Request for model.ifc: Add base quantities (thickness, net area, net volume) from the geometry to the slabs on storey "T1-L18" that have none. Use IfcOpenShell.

First a look at what the model holds.

```python
import ifcopenshell
import ifcopenshell.util.element
import ifcopenshell.util.unit

model = ifcopenshell.open("model.ifc")
print(model.schema)
for unit_type in ("LENGTHUNIT", "AREAUNIT", "VOLUMEUNIT"):
    print(unit_type, ifcopenshell.util.unit.calculate_unit_scale(model, unit_type))
storey = next(s for s in model.by_type("IfcBuildingStorey") if s.Name == "T1-L18")
slabs = [e for e in ifcopenshell.util.element.get_decomposition(storey) if e.is_a("IfcSlab")]
for e in sorted(slabs, key=lambda e: e.id()):
    print(e.id(), e.is_a(), e.Name, list(ifcopenshell.util.element.get_psets(e, qtos_only=True)), sep=" | ")
```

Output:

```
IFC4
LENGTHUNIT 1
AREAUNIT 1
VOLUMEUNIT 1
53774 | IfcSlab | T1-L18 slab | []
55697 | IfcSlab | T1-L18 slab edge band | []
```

```python
import ifcopenshell
import ifcopenshell.api.pset
import ifcopenshell.geom
import ifcopenshell.util.element
import ifcopenshell.util.shape
import ifcopenshell.util.unit

model = ifcopenshell.open("model.ifc")
unit_scale = ifcopenshell.util.unit.calculate_unit_scale(model)
area_scale = ifcopenshell.util.unit.calculate_unit_scale(model, "AREAUNIT")
volume_scale = ifcopenshell.util.unit.calculate_unit_scale(model, "VOLUMEUNIT")
settings = ifcopenshell.geom.settings()

storey = next(s for s in model.by_type("IfcBuildingStorey") if s.Name == "T1-L18")
slabs = [e for e in ifcopenshell.util.element.get_decomposition(storey) if e.is_a("IfcSlab")]

for e in sorted(slabs, key=lambda e: e.id()):
    if ifcopenshell.util.element.get_psets(e, qtos_only=True, should_inherit=False):
        continue
    # Geometry comes back in metres, in the element's own axes.
    shape = ifcopenshell.geom.create_shape(settings, e)
    values = {
        "Width": ifcopenshell.util.shape.get_z(shape.geometry) / unit_scale,
        "NetArea": ifcopenshell.util.shape.get_footprint_area(shape.geometry) / area_scale,
        "NetVolume": ifcopenshell.util.shape.get_volume(shape.geometry) / volume_scale,
    }
    qto = ifcopenshell.api.pset.add_qto(model, product=e, name="Qto_SlabBaseQuantities")
    ifcopenshell.api.pset.edit_qto(model, qto=qto, properties=values)
    print(e.id(), {k: round(v, 3) for k, v in values.items()})

model.write("model_edited.ifc")
```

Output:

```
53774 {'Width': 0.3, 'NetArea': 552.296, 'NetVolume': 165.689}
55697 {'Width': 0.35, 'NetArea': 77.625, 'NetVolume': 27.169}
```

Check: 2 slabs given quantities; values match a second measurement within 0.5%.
